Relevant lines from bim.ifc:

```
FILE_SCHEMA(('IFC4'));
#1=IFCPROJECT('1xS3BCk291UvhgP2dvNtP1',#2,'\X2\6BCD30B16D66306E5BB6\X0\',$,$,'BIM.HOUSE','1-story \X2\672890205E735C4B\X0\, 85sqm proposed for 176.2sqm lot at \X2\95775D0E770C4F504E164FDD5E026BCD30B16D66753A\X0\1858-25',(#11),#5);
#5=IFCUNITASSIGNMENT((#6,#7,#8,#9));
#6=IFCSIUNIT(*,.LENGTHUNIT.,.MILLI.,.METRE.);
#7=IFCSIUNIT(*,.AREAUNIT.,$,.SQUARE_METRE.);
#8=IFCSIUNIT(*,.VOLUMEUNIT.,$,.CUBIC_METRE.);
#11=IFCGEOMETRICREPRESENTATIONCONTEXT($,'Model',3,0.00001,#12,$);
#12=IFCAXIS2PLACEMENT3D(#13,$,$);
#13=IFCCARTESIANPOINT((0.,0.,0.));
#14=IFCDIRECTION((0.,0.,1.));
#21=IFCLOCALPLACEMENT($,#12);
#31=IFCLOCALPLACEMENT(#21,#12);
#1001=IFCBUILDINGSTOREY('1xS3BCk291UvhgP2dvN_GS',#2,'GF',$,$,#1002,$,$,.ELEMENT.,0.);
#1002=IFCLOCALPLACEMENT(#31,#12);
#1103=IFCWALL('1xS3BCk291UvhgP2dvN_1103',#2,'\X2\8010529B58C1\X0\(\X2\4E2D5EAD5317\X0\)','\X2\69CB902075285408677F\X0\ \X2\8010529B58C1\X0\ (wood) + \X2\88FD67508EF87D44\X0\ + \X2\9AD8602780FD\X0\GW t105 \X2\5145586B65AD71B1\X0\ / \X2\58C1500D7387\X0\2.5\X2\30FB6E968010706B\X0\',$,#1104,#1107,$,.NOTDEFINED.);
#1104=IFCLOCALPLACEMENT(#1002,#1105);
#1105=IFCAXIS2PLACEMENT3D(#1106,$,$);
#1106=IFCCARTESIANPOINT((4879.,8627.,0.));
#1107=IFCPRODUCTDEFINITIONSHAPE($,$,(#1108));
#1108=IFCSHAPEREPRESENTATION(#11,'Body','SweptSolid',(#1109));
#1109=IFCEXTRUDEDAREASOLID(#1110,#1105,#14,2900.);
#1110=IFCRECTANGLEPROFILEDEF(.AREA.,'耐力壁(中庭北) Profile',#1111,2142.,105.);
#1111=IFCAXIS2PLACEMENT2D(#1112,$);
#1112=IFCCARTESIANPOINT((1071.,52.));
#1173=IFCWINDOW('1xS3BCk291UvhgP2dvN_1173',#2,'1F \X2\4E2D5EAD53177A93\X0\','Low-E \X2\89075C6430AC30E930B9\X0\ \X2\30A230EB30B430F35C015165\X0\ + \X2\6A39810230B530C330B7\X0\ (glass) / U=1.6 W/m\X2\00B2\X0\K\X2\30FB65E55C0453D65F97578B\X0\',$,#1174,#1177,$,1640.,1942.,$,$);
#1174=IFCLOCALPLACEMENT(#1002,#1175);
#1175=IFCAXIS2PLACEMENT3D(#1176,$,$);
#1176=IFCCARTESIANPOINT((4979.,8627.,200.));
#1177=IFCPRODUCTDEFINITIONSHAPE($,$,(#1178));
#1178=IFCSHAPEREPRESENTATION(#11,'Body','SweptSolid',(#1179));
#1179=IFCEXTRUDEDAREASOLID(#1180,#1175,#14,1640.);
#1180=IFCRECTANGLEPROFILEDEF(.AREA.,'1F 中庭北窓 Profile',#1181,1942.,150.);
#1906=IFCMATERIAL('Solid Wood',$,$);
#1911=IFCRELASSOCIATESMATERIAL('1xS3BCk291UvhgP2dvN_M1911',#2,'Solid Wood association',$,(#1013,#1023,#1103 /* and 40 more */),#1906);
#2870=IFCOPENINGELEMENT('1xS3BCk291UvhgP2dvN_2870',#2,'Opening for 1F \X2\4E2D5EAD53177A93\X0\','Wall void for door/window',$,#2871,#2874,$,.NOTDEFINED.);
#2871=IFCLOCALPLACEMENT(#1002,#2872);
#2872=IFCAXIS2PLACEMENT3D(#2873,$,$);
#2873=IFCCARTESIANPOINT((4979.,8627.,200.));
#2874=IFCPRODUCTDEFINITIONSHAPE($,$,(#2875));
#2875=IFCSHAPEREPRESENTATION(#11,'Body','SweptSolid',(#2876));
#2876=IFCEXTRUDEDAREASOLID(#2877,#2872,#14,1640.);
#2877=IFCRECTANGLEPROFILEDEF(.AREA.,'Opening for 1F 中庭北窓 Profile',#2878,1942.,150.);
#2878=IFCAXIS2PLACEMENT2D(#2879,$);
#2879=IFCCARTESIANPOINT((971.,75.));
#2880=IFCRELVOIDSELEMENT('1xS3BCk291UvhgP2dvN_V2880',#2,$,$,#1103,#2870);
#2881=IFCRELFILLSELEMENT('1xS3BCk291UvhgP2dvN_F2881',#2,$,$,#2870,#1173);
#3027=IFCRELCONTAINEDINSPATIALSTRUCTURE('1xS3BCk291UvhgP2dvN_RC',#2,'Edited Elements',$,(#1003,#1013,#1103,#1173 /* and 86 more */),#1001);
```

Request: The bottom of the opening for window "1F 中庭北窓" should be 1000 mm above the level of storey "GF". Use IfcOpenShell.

```python
import numpy as np
import ifcopenshell
import ifcopenshell.api.geometry
import ifcopenshell.geom
import ifcopenshell.util.element
import ifcopenshell.util.placement
import ifcopenshell.util.shape
import ifcopenshell.util.unit

model = ifcopenshell.open("bim.ifc")
unit_scale = ifcopenshell.util.unit.calculate_unit_scale(model)

window = model.by_guid("1xS3BCk291UvhgP2dvN_1173")
opening = window.FillsVoids[0].RelatingOpeningElement
storey = ifcopenshell.util.element.get_container(window, ifc_class="IfcBuildingStorey")
level = ifcopenshell.util.placement.get_local_placement(storey.ObjectPlacement)[2, 3]

# The opening's origin need not be at the sill, so measure its lowest point.
shape = ifcopenshell.geom.create_shape(ifcopenshell.geom.settings(), opening)
bottom = ifcopenshell.util.shape.get_shape_bottom_elevation(shape, shape.geometry) / unit_scale
dz = level + 1 / unit_scale - bottom

shift = np.array([0.0, 0.0, dz])
# The window is not placed relative to its opening, so move both.
for product in (opening, window):
    matrix = ifcopenshell.util.placement.get_local_placement(product.ObjectPlacement)
    matrix[:3, 3] += shift
    ifcopenshell.api.geometry.edit_object_placement(model, product=product, matrix=matrix, is_si=False)

print(f"moved by {dz * unit_scale:+.3f} m")

model.write("bim_updated.ifc")
```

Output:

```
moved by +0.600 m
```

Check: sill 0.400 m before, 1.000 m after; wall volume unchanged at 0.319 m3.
